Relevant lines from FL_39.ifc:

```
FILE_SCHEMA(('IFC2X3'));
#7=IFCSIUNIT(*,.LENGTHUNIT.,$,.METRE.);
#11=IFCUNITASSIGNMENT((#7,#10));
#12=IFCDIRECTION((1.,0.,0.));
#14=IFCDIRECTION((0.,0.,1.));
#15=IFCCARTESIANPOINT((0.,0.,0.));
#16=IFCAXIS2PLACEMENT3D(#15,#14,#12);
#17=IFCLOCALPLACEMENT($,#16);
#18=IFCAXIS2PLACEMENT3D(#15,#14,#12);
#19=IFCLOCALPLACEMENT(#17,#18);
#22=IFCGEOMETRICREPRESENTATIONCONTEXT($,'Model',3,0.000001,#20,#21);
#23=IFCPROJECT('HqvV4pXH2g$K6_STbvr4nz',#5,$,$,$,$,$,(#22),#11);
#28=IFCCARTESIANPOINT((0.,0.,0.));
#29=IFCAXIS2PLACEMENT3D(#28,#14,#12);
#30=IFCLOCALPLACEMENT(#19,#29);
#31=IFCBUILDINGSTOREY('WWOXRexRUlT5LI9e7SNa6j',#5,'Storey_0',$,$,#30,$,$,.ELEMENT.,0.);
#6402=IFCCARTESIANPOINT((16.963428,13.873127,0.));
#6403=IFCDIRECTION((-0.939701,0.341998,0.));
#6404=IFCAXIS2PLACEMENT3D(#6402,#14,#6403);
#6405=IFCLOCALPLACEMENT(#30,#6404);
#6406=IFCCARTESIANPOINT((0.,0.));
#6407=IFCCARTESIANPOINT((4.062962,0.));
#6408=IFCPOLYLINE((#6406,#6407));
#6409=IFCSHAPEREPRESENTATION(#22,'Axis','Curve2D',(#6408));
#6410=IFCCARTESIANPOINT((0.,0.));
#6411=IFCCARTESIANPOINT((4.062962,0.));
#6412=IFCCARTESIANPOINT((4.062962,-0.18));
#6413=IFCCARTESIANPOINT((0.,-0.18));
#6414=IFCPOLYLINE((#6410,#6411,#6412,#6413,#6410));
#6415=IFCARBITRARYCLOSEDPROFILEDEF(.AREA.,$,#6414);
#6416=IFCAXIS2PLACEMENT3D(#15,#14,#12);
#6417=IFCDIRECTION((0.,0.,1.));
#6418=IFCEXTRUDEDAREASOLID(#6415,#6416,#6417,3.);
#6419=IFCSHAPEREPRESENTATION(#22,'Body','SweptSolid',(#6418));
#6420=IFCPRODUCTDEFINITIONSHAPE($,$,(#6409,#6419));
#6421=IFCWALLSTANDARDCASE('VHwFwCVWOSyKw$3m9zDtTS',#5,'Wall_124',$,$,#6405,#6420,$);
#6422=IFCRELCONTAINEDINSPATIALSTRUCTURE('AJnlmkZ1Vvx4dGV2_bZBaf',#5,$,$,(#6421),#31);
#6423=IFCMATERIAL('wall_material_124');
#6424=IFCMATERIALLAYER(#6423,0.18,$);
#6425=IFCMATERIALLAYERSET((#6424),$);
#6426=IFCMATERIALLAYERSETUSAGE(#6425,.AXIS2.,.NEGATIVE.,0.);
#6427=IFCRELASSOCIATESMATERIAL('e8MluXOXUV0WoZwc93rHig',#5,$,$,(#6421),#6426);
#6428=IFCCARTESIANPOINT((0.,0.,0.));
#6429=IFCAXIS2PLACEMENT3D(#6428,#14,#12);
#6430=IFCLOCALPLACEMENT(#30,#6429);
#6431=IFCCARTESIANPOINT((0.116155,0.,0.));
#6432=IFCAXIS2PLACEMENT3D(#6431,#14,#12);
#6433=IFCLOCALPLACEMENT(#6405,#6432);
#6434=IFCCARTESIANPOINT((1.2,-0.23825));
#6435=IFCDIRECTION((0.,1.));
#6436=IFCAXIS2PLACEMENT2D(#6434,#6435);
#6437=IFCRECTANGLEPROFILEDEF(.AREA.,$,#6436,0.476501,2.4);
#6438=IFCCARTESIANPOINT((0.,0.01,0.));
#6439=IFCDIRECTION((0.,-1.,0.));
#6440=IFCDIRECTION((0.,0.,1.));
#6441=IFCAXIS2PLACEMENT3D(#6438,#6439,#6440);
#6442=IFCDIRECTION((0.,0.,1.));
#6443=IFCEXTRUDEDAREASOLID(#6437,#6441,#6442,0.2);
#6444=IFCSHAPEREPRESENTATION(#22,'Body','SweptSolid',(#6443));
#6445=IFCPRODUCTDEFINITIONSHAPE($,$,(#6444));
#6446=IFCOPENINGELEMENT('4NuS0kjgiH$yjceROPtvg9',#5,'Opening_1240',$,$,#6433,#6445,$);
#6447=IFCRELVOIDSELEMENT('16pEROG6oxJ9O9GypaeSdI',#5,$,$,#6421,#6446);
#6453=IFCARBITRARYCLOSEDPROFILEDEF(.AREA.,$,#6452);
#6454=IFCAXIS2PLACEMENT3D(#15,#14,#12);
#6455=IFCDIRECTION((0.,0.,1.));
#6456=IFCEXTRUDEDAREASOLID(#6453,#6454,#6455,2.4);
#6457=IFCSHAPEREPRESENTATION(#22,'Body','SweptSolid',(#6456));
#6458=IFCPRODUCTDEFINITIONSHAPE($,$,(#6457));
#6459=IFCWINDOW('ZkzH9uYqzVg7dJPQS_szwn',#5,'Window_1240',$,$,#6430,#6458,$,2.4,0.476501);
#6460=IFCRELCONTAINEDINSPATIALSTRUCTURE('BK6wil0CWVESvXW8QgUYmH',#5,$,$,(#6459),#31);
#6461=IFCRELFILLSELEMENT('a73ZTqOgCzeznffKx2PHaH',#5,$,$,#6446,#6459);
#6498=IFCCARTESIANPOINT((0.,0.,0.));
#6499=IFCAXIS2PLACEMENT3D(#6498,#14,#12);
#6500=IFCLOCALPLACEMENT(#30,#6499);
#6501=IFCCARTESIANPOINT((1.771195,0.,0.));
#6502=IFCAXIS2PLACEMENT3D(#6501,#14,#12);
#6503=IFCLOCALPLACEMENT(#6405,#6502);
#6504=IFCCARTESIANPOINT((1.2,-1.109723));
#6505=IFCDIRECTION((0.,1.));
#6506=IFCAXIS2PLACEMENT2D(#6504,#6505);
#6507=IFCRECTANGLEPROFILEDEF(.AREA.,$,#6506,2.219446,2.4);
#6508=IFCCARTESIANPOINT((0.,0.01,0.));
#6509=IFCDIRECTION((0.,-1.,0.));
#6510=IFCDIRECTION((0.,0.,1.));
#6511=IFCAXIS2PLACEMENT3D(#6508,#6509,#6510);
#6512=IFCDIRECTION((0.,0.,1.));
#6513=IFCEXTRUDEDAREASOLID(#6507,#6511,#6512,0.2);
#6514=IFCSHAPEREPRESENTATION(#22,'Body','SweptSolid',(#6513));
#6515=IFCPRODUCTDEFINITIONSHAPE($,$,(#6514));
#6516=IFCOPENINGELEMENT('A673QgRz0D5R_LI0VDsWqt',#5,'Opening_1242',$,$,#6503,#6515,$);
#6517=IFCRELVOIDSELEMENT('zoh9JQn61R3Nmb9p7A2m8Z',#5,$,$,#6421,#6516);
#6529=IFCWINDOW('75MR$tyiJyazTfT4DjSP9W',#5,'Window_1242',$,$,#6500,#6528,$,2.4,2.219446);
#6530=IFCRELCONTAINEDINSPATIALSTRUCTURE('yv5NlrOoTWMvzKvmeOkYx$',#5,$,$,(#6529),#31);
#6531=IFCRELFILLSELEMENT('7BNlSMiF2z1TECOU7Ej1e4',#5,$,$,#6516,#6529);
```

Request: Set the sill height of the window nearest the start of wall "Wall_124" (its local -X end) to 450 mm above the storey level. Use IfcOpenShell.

```python
import numpy as np
import ifcopenshell
import ifcopenshell.api.geometry
import ifcopenshell.geom
import ifcopenshell.util.element
import ifcopenshell.util.placement
import ifcopenshell.util.shape
import ifcopenshell.util.unit

model = ifcopenshell.open("FL_39.ifc")
unit_scale = ifcopenshell.util.unit.calculate_unit_scale(model)

window = model.by_id(6459)
opening = window.FillsVoids[0].RelatingOpeningElement
storey = ifcopenshell.util.element.get_container(window, ifc_class="IfcBuildingStorey")
level = ifcopenshell.util.placement.get_local_placement(storey.ObjectPlacement)[2, 3]

# The opening's origin need not be at the sill, so measure its lowest point.
shape = ifcopenshell.geom.create_shape(ifcopenshell.geom.settings(), opening)
bottom = ifcopenshell.util.shape.get_shape_bottom_elevation(shape, shape.geometry) / unit_scale
dz = level + 0.45 / unit_scale - bottom

shift = np.array([0.0, 0.0, dz])
# The window is not placed relative to its opening, so move both.
for product in (opening, window):
    matrix = ifcopenshell.util.placement.get_local_placement(product.ObjectPlacement)
    matrix[:3, 3] += shift
    ifcopenshell.api.geometry.edit_object_placement(model, product=product, matrix=matrix, is_si=False)

print(f"moved by {dz * unit_scale:+.3f} m")

model.write("FL_39_rev.ifc")
```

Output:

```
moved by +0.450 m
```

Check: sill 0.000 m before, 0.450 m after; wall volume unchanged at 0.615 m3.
